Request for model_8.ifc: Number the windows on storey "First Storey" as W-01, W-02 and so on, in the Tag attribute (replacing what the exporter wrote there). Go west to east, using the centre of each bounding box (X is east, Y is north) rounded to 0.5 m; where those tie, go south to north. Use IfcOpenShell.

First a look at what the model holds.

```python
import ifcopenshell
import ifcopenshell.util.element
import ifcopenshell.util.placement

model = ifcopenshell.open("model_8.ifc")
print(model.schema)
storey = next(s for s in model.by_type("IfcBuildingStorey") if s.Name == "First Storey")
windows = [e for e in ifcopenshell.util.element.get_decomposition(storey) if e.is_a("IfcWindow")]
for e in sorted(windows, key=lambda e: e.id()):
    origin = ifcopenshell.util.placement.get_local_placement(e.ObjectPlacement)[:3, 3]
    print(e.id(), e.Tag, e.Name, origin.round(2) + 0.0, sep=" | ")
```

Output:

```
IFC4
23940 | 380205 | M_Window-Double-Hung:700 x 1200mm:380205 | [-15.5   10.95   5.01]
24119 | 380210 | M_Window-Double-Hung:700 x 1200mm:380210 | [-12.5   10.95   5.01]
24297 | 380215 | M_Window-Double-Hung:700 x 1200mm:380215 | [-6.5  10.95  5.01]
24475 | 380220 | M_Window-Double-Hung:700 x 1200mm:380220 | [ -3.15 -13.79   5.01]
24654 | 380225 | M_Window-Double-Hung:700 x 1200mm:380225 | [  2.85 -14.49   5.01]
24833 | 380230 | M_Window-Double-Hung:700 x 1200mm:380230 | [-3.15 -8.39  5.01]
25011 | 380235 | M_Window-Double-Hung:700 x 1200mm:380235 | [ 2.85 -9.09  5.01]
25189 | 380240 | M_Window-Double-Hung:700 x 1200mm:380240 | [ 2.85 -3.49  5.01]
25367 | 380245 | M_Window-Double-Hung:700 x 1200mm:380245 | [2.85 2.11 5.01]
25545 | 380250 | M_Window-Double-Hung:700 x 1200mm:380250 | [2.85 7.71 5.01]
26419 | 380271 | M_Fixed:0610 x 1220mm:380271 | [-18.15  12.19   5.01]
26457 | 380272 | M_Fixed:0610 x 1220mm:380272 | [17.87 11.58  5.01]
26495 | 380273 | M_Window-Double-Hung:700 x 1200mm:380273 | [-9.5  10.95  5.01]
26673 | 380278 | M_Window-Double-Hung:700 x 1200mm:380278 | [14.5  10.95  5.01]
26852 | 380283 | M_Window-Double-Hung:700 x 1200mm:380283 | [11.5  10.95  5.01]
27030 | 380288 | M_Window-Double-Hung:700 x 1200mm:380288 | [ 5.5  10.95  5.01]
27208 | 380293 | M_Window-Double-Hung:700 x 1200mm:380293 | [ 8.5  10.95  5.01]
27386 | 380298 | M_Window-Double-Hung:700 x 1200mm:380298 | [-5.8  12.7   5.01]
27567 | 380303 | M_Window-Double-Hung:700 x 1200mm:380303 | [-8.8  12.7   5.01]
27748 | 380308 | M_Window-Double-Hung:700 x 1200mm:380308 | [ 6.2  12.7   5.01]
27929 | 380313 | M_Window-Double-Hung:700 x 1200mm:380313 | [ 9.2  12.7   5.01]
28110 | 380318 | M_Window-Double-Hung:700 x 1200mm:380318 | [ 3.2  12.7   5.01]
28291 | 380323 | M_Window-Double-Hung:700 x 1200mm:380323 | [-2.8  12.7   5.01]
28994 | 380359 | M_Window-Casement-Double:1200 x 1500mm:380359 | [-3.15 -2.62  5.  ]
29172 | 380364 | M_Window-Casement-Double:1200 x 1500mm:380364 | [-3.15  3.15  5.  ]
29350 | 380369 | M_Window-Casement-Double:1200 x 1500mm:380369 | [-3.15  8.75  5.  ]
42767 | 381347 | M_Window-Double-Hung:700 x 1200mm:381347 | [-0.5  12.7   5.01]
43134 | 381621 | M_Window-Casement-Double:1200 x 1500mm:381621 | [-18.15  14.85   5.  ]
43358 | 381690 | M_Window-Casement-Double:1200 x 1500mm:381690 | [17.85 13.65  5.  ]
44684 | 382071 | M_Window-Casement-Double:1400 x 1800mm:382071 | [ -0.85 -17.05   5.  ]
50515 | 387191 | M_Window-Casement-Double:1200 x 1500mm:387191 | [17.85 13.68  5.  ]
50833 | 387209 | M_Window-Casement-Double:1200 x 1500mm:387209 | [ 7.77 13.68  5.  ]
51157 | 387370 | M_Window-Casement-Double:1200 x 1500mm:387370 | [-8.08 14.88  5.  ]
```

```python
import ifcopenshell
import ifcopenshell.geom
import ifcopenshell.util.element
import ifcopenshell.util.shape

model = ifcopenshell.open("model_8.ifc")
settings = ifcopenshell.geom.settings()
settings.set("use-world-coords", True)


def centre(element):
    shape = ifcopenshell.geom.create_shape(settings, element)
    return ifcopenshell.util.shape.get_bbox_centroid(shape.geometry)


storey = next(s for s in model.by_type("IfcBuildingStorey") if s.Name == "First Storey")
windows = [e for e in ifcopenshell.util.element.get_decomposition(storey) if e.is_a("IfcWindow")]

# Insertion points can sit at a corner or the storey origin, so sort by the geometry (in metres).
centres = {e: centre(e) for e in windows}
windows.sort(key=lambda e: (round(centres[e][0] / 0.5), centres[e][1]))

for i, e in enumerate(windows, start=1):
    number = f"W-{i:02d}"
    e.Tag = number
    print(e.id(), number)

model.write("model_8_v2.ifc")
```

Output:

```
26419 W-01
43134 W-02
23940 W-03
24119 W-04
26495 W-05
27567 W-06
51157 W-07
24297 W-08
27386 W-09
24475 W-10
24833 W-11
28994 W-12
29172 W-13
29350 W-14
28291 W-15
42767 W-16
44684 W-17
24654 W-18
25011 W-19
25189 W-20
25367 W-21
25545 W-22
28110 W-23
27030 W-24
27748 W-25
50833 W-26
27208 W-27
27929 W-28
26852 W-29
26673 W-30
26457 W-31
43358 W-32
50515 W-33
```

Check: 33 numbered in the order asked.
